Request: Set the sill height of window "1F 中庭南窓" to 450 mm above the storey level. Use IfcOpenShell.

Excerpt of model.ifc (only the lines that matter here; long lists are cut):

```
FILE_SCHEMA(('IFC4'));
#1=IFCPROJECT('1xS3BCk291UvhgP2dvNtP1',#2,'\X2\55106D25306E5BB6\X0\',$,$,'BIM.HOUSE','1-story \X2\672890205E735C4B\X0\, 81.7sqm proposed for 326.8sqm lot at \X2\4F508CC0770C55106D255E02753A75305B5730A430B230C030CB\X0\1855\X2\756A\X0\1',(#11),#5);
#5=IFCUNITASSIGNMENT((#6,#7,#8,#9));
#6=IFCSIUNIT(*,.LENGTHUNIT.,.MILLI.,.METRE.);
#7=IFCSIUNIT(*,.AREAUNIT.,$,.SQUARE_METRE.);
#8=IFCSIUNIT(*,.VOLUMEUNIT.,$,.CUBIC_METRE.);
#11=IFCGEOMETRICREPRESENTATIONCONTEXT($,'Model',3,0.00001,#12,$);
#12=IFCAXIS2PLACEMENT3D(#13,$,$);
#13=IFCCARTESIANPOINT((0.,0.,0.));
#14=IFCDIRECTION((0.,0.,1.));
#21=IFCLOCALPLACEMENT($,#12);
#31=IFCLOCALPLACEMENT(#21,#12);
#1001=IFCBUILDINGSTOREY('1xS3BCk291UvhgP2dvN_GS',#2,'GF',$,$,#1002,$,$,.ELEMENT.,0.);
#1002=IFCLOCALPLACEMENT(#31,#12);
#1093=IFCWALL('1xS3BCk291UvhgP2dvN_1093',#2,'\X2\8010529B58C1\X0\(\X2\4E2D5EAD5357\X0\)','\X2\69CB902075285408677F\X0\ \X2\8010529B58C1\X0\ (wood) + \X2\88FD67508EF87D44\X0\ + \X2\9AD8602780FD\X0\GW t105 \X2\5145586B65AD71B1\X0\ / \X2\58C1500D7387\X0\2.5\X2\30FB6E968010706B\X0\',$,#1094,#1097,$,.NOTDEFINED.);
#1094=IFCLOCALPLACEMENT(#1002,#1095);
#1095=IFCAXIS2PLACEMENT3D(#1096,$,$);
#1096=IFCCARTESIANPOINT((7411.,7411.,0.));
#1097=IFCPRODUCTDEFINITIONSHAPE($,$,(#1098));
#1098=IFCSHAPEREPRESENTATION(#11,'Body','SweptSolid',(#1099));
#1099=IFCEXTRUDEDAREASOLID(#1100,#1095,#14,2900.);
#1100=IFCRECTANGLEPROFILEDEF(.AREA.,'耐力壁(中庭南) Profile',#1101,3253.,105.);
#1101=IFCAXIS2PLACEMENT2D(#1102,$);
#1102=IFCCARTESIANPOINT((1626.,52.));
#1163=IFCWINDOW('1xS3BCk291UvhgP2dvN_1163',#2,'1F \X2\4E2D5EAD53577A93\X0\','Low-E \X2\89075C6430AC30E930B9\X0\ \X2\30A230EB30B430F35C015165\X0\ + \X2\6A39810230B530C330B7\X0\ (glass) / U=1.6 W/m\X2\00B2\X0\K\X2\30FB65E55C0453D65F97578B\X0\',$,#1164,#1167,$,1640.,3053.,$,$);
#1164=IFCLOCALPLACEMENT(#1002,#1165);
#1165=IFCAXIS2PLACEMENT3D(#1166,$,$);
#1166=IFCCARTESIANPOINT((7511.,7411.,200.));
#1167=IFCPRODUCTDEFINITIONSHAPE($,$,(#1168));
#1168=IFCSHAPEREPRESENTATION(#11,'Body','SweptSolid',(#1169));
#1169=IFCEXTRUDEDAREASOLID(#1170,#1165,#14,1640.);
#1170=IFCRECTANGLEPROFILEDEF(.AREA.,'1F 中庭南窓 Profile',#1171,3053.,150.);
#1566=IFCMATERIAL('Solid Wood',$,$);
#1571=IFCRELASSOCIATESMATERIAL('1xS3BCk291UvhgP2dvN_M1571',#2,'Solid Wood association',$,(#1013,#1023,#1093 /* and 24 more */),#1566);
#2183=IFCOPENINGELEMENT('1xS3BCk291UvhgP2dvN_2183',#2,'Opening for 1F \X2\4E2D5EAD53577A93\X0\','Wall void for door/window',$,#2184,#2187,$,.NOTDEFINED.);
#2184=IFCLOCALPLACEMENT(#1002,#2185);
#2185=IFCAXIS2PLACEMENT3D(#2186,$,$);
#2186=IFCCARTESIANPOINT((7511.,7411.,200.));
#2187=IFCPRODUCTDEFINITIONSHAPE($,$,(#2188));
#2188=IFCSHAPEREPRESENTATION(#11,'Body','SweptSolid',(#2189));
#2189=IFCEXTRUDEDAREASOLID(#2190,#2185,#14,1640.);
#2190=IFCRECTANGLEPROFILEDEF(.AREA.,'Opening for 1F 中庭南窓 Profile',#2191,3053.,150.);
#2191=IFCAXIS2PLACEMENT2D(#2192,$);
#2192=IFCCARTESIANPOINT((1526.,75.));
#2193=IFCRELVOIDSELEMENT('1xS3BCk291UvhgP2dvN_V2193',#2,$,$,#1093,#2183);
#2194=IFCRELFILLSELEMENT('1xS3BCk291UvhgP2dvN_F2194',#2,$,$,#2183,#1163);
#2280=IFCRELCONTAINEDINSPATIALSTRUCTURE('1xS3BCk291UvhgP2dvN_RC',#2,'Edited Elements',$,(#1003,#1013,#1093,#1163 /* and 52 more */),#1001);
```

```python
import numpy as np
import ifcopenshell
import ifcopenshell.api.geometry
import ifcopenshell.geom
import ifcopenshell.util.element
import ifcopenshell.util.placement
import ifcopenshell.util.shape
import ifcopenshell.util.unit

model = ifcopenshell.open("model.ifc")
unit_scale = ifcopenshell.util.unit.calculate_unit_scale(model)

window = model.by_guid("1xS3BCk291UvhgP2dvN_1163")
opening = window.FillsVoids[0].RelatingOpeningElement
storey = ifcopenshell.util.element.get_container(window, ifc_class="IfcBuildingStorey")
level = ifcopenshell.util.placement.get_local_placement(storey.ObjectPlacement)[2, 3]

# The opening's origin need not be at the sill, so measure its lowest point.
shape = ifcopenshell.geom.create_shape(ifcopenshell.geom.settings(), opening)
bottom = ifcopenshell.util.shape.get_shape_bottom_elevation(shape, shape.geometry) / unit_scale
dz = level + 450.0 - bottom

shift = np.array([0.0, 0.0, dz])
# The window is not placed relative to its opening, so move both.
for product in (opening, window):
    matrix = ifcopenshell.util.placement.get_local_placement(product.ObjectPlacement)
    matrix[:3, 3] += shift
    ifcopenshell.api.geometry.edit_object_placement(model, product=product, matrix=matrix, is_si=False)

print(f"moved by {dz * unit_scale:+.3f} m")

model.write("model_rev.ifc")
```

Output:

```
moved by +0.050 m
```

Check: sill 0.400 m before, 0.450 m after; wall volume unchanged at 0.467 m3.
